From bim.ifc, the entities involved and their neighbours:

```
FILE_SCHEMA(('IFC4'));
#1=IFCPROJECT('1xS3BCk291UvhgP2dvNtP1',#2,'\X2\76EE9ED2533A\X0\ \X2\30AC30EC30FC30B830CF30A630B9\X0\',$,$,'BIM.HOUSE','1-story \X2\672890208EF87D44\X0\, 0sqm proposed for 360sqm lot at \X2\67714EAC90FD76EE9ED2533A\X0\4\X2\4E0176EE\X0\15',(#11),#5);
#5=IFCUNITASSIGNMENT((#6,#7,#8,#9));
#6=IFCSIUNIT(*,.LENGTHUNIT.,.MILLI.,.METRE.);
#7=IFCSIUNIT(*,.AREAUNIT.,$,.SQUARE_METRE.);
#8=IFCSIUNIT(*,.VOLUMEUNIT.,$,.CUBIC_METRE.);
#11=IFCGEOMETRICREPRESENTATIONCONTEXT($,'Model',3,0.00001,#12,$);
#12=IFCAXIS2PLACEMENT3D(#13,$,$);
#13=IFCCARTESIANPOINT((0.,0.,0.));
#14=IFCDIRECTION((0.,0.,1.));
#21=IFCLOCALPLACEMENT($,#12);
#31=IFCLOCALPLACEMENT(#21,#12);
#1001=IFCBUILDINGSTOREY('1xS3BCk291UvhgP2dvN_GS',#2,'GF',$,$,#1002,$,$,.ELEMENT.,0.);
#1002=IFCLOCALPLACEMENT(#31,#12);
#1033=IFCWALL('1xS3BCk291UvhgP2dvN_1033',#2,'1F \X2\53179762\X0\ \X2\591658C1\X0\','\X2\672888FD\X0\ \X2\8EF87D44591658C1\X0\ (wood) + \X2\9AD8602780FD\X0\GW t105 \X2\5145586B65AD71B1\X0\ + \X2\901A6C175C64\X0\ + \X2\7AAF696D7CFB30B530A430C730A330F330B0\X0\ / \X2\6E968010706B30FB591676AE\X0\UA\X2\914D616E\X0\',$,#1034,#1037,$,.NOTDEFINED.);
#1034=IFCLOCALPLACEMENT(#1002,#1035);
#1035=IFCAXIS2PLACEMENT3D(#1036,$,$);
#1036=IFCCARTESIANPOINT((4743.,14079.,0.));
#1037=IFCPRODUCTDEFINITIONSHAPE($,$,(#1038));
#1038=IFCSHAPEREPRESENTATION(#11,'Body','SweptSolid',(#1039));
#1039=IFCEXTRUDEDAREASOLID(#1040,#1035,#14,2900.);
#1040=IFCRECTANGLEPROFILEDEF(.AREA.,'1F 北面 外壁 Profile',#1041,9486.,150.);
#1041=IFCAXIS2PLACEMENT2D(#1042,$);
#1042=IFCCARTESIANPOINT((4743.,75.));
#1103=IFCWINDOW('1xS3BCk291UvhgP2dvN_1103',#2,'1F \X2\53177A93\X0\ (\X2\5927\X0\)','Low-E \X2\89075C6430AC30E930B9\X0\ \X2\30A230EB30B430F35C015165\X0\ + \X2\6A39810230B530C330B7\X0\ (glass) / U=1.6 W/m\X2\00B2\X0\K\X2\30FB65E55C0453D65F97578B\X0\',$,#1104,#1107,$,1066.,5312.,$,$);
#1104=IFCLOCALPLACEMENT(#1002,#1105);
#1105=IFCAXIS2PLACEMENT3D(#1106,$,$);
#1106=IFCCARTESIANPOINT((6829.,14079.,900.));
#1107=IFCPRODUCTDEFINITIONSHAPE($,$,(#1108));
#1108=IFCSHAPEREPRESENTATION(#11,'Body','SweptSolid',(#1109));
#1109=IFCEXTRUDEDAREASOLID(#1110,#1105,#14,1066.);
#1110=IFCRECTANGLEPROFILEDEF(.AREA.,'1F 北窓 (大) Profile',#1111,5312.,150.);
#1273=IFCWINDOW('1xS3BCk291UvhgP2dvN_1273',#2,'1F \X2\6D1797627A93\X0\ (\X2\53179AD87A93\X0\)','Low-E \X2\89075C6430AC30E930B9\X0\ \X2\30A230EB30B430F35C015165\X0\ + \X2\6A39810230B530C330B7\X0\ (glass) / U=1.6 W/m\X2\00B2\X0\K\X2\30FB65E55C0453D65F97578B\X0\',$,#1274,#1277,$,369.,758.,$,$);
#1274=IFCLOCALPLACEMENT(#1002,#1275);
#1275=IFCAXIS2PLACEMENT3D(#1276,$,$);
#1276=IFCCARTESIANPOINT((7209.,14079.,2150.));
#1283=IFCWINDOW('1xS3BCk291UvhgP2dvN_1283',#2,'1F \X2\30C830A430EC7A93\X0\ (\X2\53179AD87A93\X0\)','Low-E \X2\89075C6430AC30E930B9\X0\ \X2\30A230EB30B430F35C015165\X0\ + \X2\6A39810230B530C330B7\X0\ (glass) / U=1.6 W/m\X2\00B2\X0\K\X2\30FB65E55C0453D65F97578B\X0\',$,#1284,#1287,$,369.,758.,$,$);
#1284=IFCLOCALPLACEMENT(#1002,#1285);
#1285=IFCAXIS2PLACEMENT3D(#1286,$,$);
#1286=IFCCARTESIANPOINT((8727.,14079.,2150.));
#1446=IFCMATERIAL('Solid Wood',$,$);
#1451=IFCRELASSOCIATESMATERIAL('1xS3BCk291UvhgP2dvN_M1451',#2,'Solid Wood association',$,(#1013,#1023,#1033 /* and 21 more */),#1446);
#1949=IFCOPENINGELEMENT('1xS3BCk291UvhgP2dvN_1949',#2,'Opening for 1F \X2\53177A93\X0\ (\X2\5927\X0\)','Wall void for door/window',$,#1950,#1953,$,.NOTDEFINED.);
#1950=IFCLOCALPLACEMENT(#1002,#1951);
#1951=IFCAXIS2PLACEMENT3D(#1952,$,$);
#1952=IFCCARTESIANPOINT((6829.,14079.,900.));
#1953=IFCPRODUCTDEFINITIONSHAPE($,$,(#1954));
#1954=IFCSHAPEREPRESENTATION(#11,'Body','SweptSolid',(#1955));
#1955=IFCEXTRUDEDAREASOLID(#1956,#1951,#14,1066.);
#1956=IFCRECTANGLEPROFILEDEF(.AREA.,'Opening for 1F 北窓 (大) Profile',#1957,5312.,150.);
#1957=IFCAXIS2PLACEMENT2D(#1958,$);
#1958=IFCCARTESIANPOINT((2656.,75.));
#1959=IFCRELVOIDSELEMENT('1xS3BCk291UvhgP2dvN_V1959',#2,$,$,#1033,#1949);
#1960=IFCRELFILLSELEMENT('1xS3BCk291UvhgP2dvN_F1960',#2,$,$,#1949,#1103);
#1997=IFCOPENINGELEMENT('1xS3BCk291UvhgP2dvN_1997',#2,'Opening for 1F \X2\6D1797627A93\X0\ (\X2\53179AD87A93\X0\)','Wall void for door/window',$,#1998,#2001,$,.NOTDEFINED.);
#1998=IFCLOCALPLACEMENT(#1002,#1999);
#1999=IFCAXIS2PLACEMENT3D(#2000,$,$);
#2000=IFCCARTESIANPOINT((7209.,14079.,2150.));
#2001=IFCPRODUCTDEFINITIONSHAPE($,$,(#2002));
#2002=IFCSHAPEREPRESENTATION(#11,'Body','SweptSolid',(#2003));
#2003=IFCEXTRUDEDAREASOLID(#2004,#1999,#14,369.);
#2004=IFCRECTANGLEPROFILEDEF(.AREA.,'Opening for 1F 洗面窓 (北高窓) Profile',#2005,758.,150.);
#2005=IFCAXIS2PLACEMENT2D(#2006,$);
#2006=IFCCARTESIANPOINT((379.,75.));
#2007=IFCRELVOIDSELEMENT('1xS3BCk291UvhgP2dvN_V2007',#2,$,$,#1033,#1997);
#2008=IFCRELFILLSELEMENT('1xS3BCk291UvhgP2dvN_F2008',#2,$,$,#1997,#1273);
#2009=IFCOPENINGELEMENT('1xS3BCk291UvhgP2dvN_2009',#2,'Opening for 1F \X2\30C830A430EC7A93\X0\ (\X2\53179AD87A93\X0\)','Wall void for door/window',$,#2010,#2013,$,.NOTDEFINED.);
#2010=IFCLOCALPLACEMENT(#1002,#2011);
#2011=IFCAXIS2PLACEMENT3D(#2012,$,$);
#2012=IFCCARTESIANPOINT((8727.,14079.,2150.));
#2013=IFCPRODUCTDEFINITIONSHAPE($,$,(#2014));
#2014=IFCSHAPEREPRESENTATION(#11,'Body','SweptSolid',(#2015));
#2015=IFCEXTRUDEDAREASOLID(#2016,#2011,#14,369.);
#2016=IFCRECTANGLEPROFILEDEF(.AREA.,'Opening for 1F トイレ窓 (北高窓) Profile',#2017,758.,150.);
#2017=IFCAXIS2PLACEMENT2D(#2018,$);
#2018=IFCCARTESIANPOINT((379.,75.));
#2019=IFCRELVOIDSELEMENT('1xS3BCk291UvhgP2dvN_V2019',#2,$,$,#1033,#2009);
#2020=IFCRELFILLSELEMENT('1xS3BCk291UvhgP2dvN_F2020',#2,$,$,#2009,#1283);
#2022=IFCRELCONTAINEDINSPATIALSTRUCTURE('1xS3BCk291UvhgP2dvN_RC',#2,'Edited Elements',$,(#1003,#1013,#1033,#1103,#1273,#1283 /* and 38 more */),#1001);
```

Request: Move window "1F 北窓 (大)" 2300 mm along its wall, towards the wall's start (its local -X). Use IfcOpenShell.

```python
import ifcopenshell
import ifcopenshell.api.geometry
import ifcopenshell.util.placement
import ifcopenshell.util.unit

model = ifcopenshell.open("bim.ifc")
unit_scale = ifcopenshell.util.unit.calculate_unit_scale(model)

window = model.by_guid("1xS3BCk291UvhgP2dvN_1103")
opening = window.FillsVoids[0].RelatingOpeningElement
wall = opening.VoidsElements[0].RelatingBuildingElement

wall_matrix = ifcopenshell.util.placement.get_local_placement(wall.ObjectPlacement)
shift = wall_matrix[:3, 0] * -2.3 / unit_scale
before = ifcopenshell.util.placement.get_local_placement(window.ObjectPlacement)[:3, 3].copy()

# The window is not placed relative to its opening, so move both.
for product in (opening, window):
    matrix = ifcopenshell.util.placement.get_local_placement(product.ObjectPlacement)
    matrix[:3, 3] += shift
    ifcopenshell.api.geometry.edit_object_placement(model, product=product, matrix=matrix, is_si=False)

after = ifcopenshell.util.placement.get_local_placement(window.ObjectPlacement)[:3, 3]
print("window moved by", (after - before).round(3) + 0.0)

model.write("bim-out.ifc")
```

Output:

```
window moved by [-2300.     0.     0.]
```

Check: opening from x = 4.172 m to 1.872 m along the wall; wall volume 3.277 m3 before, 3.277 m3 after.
